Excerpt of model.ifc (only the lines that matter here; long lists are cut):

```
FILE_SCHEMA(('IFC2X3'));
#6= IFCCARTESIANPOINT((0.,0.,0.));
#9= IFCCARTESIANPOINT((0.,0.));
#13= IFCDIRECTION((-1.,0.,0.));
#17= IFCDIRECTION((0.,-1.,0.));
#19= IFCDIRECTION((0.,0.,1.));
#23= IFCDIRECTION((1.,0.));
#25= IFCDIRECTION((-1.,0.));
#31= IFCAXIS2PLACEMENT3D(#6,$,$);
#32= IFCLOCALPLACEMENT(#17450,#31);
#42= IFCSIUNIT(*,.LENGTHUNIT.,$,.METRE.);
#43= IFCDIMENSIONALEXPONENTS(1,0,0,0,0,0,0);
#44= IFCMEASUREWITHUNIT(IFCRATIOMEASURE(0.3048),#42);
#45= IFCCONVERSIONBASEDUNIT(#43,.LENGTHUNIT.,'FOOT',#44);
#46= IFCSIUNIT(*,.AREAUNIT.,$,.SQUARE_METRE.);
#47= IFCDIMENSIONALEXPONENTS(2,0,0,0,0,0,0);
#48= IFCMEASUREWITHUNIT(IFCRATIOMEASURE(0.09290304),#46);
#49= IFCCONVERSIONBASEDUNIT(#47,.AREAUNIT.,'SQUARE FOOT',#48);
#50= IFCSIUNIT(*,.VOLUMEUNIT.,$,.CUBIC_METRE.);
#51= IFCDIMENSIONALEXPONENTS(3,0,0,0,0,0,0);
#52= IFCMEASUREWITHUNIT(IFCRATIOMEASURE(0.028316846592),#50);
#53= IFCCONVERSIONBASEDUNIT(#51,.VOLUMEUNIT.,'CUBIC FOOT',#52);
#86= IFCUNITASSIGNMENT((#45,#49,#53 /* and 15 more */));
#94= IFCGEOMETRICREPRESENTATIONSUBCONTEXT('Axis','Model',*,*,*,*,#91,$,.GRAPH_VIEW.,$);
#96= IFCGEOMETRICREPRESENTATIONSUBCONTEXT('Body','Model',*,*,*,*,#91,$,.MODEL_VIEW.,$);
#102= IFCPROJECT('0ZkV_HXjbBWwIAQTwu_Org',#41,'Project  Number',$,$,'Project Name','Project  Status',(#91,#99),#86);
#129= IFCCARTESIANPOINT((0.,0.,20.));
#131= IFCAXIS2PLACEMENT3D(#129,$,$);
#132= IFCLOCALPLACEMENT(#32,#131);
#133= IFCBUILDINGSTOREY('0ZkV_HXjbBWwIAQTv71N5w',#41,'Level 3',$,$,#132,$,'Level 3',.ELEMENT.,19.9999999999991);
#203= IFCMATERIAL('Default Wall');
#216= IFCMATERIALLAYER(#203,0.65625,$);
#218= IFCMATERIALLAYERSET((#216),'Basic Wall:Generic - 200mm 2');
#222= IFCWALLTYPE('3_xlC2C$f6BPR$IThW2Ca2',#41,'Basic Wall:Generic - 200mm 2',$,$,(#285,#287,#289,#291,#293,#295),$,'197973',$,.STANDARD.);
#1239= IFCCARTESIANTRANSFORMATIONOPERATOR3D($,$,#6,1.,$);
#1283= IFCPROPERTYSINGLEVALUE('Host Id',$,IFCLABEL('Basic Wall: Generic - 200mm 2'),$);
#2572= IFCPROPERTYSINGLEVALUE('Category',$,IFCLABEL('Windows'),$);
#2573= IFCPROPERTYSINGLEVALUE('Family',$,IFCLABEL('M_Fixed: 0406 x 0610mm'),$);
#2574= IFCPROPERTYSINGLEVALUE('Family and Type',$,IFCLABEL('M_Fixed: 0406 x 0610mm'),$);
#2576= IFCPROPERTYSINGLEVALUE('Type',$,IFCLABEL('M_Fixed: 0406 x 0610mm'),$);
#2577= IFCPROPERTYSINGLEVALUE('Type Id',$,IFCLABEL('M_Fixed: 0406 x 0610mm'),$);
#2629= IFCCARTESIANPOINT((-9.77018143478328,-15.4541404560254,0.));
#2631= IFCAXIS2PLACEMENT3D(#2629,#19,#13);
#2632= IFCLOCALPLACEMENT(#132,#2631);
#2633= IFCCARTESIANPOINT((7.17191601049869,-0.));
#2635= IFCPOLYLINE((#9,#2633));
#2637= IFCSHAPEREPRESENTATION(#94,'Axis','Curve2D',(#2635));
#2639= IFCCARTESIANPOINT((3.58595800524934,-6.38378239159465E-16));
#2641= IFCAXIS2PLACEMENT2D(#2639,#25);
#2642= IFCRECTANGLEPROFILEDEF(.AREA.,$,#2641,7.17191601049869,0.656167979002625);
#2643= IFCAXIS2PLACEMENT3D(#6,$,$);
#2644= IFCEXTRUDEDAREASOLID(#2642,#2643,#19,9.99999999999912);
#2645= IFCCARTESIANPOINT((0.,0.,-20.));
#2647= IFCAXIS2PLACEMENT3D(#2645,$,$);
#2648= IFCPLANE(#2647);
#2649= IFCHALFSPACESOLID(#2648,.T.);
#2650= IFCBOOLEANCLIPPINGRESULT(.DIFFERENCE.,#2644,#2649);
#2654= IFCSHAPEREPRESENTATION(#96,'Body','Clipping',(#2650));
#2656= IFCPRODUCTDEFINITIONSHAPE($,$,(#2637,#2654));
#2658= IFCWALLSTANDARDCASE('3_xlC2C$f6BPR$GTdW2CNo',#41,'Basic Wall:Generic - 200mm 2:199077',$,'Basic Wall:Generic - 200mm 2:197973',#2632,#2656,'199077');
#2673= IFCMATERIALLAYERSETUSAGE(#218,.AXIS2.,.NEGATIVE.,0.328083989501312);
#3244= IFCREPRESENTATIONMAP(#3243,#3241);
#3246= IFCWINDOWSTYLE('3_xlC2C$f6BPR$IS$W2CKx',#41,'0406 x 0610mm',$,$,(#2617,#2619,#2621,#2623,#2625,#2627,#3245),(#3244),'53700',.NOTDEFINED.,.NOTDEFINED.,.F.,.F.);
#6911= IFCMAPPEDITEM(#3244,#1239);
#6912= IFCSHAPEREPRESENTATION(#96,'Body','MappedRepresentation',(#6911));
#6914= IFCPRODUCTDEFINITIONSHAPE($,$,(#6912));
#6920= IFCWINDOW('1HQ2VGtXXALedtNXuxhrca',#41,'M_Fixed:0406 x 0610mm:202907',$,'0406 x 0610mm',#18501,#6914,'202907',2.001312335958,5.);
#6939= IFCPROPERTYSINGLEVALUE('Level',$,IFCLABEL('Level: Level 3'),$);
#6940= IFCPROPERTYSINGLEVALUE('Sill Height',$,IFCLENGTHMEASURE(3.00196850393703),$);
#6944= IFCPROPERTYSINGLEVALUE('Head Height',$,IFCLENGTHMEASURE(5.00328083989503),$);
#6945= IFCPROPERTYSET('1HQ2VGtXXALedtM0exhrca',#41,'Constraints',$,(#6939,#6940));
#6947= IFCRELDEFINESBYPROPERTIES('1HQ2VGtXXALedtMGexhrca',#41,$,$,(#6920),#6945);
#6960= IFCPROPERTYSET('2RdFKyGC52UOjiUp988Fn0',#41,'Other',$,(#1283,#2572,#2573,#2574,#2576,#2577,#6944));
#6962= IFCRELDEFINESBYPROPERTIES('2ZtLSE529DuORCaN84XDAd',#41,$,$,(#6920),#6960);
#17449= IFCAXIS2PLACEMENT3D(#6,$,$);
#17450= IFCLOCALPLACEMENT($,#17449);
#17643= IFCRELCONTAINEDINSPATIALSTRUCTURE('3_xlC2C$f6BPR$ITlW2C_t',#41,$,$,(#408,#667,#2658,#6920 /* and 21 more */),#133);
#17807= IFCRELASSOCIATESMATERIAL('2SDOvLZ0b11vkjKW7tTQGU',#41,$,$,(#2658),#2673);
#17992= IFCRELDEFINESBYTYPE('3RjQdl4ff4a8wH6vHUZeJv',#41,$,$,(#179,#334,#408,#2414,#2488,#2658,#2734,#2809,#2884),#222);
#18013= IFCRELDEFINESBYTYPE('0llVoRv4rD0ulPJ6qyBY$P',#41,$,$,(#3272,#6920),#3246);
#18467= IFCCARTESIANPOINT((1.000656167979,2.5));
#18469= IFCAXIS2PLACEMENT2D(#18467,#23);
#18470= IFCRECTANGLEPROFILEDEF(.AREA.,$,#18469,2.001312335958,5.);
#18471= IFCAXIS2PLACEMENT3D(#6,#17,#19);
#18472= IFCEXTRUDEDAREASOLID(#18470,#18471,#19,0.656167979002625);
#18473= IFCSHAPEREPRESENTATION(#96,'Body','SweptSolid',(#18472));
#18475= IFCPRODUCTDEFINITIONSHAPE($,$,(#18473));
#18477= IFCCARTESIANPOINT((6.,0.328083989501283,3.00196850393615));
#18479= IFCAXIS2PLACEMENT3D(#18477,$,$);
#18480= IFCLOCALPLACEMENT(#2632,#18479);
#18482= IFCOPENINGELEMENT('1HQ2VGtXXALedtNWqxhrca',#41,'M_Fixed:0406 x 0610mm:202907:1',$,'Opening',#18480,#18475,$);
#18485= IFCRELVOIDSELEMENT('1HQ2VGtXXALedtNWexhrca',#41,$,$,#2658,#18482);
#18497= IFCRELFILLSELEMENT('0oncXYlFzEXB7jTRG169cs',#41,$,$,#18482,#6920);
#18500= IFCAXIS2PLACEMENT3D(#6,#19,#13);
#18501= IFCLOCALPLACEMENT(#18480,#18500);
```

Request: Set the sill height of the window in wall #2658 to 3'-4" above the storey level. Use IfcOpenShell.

```python
import numpy as np
import ifcopenshell
import ifcopenshell.api.geometry
import ifcopenshell.api.pset
import ifcopenshell.geom
import ifcopenshell.util.element
import ifcopenshell.util.placement
import ifcopenshell.util.shape
import ifcopenshell.util.unit

model = ifcopenshell.open("model.ifc")
unit_scale = ifcopenshell.util.unit.calculate_unit_scale(model)

window = model.by_guid("1HQ2VGtXXALedtNXuxhrca")
opening = window.FillsVoids[0].RelatingOpeningElement
storey = ifcopenshell.util.element.get_container(window, ifc_class="IfcBuildingStorey")
level = ifcopenshell.util.placement.get_local_placement(storey.ObjectPlacement)[2, 3]

# The opening's origin need not be at the sill, so measure its lowest point.
shape = ifcopenshell.geom.create_shape(ifcopenshell.geom.settings(), opening)
bottom = ifcopenshell.util.shape.get_shape_bottom_elevation(shape, shape.geometry) / unit_scale
dz = level + 40 * 0.0254 / unit_scale - bottom

shift = np.array([0.0, 0.0, dz])
# The window is placed relative to its opening, so it follows when the opening moves.
matrix = ifcopenshell.util.placement.get_local_placement(opening.ObjectPlacement)
matrix[:3, 3] += shift
ifcopenshell.api.geometry.edit_object_placement(
    model, product=opening, matrix=matrix, is_si=False, should_transform_children=True
)

# Keep the stored heights in step.
pset = model.by_id(ifcopenshell.util.element.get_pset(window, "Constraints", should_inherit=False)["id"])
ifcopenshell.api.pset.edit_pset(model, pset=pset, properties={
    "Sill Height": model.create_entity("IfcLengthMeasure", ifcopenshell.util.element.get_pset(window, "Constraints", "Sill Height") + dz),
})
pset = model.by_id(ifcopenshell.util.element.get_pset(window, "Other", should_inherit=False)["id"])
ifcopenshell.api.pset.edit_pset(model, pset=pset, properties={
    "Head Height": model.create_entity("IfcLengthMeasure", ifcopenshell.util.element.get_pset(window, "Other", "Head Height") + dz),
})

print(f"moved by {dz * unit_scale:+.3f} m")

model.write("model-out.ifc")
```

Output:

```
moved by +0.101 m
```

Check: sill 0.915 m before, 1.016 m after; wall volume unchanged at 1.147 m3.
